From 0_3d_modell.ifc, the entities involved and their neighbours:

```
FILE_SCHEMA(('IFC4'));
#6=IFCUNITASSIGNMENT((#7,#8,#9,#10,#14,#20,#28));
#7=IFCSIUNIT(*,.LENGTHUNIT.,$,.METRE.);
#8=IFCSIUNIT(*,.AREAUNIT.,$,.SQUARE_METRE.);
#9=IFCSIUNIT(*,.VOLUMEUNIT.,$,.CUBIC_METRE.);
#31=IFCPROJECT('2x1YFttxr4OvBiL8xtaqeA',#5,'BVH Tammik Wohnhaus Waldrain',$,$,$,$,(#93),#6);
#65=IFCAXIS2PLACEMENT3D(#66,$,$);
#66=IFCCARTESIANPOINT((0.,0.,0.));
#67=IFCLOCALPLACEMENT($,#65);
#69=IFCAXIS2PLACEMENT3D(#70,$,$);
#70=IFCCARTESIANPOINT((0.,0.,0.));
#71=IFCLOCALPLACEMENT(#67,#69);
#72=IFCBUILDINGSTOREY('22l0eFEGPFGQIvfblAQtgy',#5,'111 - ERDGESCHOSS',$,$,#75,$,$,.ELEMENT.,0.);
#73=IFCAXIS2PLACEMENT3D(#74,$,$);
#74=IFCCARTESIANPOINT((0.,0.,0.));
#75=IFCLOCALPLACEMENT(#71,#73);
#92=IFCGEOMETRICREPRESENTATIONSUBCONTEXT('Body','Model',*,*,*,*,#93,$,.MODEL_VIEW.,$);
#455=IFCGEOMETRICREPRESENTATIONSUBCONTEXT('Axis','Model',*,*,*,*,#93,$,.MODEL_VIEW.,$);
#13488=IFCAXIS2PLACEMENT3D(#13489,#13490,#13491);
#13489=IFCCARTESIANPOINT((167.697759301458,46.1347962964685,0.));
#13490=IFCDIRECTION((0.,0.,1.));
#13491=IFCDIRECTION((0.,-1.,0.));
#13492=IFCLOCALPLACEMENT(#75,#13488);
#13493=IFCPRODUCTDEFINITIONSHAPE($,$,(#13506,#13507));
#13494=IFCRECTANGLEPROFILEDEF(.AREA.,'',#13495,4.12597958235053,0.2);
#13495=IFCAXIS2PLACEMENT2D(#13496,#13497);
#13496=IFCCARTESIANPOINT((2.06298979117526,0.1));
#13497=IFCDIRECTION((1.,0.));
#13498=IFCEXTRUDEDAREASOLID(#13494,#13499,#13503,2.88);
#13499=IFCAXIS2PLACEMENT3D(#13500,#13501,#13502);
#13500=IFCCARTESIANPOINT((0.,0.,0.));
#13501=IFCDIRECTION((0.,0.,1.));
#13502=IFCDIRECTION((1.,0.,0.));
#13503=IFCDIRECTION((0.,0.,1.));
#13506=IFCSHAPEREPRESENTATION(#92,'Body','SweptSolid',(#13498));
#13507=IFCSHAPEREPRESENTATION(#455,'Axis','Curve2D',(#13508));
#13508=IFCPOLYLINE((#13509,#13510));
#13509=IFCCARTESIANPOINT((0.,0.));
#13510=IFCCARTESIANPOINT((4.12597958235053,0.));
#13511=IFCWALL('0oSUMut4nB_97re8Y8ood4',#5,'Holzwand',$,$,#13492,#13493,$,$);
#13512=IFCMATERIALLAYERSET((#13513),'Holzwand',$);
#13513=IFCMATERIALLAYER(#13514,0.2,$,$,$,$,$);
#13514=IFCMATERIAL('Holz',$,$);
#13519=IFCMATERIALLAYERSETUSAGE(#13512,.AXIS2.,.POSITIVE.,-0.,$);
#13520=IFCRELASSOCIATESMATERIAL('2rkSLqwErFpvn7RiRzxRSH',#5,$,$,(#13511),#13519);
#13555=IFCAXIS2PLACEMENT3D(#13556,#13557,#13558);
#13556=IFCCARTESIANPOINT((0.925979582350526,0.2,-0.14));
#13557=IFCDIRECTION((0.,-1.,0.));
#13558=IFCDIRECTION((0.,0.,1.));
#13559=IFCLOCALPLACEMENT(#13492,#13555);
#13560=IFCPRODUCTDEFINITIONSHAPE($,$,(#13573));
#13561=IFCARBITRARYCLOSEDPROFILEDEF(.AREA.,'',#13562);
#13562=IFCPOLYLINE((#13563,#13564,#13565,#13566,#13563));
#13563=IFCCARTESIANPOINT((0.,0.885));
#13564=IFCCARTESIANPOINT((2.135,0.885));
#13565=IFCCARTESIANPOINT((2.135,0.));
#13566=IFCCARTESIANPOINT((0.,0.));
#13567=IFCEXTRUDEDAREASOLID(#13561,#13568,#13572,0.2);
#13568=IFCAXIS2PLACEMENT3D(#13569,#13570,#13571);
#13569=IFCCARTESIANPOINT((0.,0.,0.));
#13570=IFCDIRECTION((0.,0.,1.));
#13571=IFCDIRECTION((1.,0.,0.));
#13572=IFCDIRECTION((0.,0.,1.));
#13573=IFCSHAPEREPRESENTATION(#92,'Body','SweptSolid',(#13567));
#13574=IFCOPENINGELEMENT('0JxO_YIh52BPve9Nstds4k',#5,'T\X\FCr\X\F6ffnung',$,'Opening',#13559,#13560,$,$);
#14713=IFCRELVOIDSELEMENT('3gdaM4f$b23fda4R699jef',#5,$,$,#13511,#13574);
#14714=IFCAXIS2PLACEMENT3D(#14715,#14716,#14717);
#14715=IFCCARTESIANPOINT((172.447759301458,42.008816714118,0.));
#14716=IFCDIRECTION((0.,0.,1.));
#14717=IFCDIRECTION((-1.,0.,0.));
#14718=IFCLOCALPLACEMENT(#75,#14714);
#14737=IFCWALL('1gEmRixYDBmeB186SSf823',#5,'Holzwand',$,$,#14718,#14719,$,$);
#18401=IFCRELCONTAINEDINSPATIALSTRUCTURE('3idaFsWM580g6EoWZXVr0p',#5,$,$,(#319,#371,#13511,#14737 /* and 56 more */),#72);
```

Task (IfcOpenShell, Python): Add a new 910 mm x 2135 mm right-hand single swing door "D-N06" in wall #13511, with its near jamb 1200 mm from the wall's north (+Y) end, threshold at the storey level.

```python
import numpy as np
import ifcopenshell
import ifcopenshell.api.feature
import ifcopenshell.api.geometry
import ifcopenshell.api.root
import ifcopenshell.api.spatial
import ifcopenshell.geom
import ifcopenshell.util.element
import ifcopenshell.util.placement
import ifcopenshell.util.representation
import ifcopenshell.util.shape
import ifcopenshell.util.unit

model = ifcopenshell.open("0_3d_modell.ifc")
unit_scale = ifcopenshell.util.unit.calculate_unit_scale(model)
settings = ifcopenshell.geom.settings()


def volume(element):
    """Net volume in cubic metres, openings subtracted."""
    shape = ifcopenshell.geom.create_shape(settings, element)
    return ifcopenshell.util.shape.get_volume(shape.geometry)


wall = model.by_guid("0oSUMut4nB_97re8Y8ood4")
storey = ifcopenshell.util.element.get_container(wall, ifc_class="IfcBuildingStorey")
context = ifcopenshell.util.representation.get_context(model, "Model", "Body", "MODEL_VIEW")
before = volume(wall)

width, height, from_end, sill = 0.91, 2.135, 1.2, 0.0  # metres

# The wall runs along its own X axis, and the end named is its -X end.
wall_shape = ifcopenshell.geom.create_shape(settings, wall)
x, y, z = ifcopenshell.util.shape.get_vertices(wall_shape.geometry).T
start = x.min() + from_end
face, thickness = float(y.min()), float(y.max() - y.min())
wall_matrix = ifcopenshell.util.placement.get_local_placement(wall.ObjectPlacement)
level = ifcopenshell.util.placement.get_local_placement(storey.ObjectPlacement)[2, 3]


def in_wall(x, y):
    """Placement at x, y metres in the wall's axes, at sill height."""
    matrix = wall_matrix.copy()
    matrix[:, 3] = wall_matrix @ np.array([x / unit_scale, y / unit_scale, 0.0, 1.0])
    matrix[2, 3] = level + sill / unit_scale
    return matrix


# Opening: a box that overshoots both wall faces by 50 mm.
opening = ifcopenshell.api.root.create_entity(model, ifc_class="IfcOpeningElement", predefined_type="OPENING")
box = ifcopenshell.api.geometry.add_wall_representation(
    model, context=context, length=width, height=height, thickness=thickness + 0.1
)
ifcopenshell.api.geometry.assign_representation(model, product=opening, representation=box)
ifcopenshell.api.geometry.edit_object_placement(model, product=opening, matrix=in_wall(start, face - 0.05), is_si=False)
ifcopenshell.api.feature.add_feature(model, feature=opening, element=wall)

door = ifcopenshell.api.root.create_entity(model, ifc_class="IfcDoor", name="D-N06", predefined_type="DOOR")
door.OverallWidth, door.OverallHeight = width / unit_scale, height / unit_scale
door.OperationType = "SINGLE_SWING_RIGHT"
body = ifcopenshell.api.geometry.add_door_representation(
    model,
    context=context,
    overall_width=door.OverallWidth,
    overall_height=door.OverallHeight,
    operation_type="SINGLE_SWING_RIGHT",
    lining_properties={"LiningDepth": thickness / unit_scale, "ThresholdDepth": thickness / unit_scale},
)
ifcopenshell.api.geometry.assign_representation(model, product=door, representation=body)
ifcopenshell.api.spatial.assign_container(model, products=[door], relating_structure=storey)
ifcopenshell.api.feature.add_filling(model, opening=opening, element=door)

# The lining spans the wall, so the door starts at the wall face.
ifcopenshell.api.geometry.edit_object_placement(model, product=door, matrix=in_wall(start, face), is_si=False)

after = volume(wall)

print(f"wall volume {before:.3f} -> {after:.3f} m3")

model.write("0_3d_modell_updated.ifc")
```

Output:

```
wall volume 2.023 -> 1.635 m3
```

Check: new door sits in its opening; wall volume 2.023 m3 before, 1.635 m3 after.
